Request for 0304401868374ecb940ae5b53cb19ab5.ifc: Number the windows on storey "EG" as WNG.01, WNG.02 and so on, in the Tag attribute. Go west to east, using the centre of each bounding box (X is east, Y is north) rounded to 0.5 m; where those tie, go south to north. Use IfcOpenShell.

First a look at what the model holds.

```python
import ifcopenshell
import ifcopenshell.util.element
import ifcopenshell.util.placement

model = ifcopenshell.open("0304401868374ecb940ae5b53cb19ab5.ifc")
print(model.schema)
storey = next(s for s in model.by_type("IfcBuildingStorey") if s.Name == "EG")
windows = [e for e in ifcopenshell.util.element.get_decomposition(storey) if e.is_a("IfcWindow")]
for e in sorted(windows, key=lambda e: e.id()):
    origin = ifcopenshell.util.placement.get_local_placement(e.ObjectPlacement)[:3, 3]
    print(e.id(), e.Tag, e.Name, origin.round(2) + 0.0, sep=" | ")
```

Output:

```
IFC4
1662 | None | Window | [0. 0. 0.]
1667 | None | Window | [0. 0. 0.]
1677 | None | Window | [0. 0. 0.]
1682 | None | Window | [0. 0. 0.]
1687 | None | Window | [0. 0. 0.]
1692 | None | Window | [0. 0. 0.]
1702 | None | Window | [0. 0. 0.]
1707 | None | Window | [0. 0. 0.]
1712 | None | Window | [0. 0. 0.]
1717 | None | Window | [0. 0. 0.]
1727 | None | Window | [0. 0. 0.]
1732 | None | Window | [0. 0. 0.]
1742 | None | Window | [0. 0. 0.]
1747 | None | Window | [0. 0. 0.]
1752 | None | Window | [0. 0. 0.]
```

```python
import ifcopenshell
import ifcopenshell.geom
import ifcopenshell.util.element
import ifcopenshell.util.shape

model = ifcopenshell.open("0304401868374ecb940ae5b53cb19ab5.ifc")
settings = ifcopenshell.geom.settings()
settings.set("use-world-coords", True)


def centre(element):
    shape = ifcopenshell.geom.create_shape(settings, element)
    return ifcopenshell.util.shape.get_bbox_centroid(shape.geometry)


storey = next(s for s in model.by_type("IfcBuildingStorey") if s.Name == "EG")
windows = [e for e in ifcopenshell.util.element.get_decomposition(storey) if e.is_a("IfcWindow")]

# Insertion points can sit at a corner or the storey origin, so sort by the geometry (in metres).
centres = {e: centre(e) for e in windows}
windows.sort(key=lambda e: (round(centres[e][0] / 0.5), centres[e][1]))

for i, e in enumerate(windows, start=1):
    number = f"WNG.{i:02d}"
    e.Tag = number
    print(e.id(), number)

model.write("0304401868374ecb940ae5b53cb19ab5_edited.ifc")
```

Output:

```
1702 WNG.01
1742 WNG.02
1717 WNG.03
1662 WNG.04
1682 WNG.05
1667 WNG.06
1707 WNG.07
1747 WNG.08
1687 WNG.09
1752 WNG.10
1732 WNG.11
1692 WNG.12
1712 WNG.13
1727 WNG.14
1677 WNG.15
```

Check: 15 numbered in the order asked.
